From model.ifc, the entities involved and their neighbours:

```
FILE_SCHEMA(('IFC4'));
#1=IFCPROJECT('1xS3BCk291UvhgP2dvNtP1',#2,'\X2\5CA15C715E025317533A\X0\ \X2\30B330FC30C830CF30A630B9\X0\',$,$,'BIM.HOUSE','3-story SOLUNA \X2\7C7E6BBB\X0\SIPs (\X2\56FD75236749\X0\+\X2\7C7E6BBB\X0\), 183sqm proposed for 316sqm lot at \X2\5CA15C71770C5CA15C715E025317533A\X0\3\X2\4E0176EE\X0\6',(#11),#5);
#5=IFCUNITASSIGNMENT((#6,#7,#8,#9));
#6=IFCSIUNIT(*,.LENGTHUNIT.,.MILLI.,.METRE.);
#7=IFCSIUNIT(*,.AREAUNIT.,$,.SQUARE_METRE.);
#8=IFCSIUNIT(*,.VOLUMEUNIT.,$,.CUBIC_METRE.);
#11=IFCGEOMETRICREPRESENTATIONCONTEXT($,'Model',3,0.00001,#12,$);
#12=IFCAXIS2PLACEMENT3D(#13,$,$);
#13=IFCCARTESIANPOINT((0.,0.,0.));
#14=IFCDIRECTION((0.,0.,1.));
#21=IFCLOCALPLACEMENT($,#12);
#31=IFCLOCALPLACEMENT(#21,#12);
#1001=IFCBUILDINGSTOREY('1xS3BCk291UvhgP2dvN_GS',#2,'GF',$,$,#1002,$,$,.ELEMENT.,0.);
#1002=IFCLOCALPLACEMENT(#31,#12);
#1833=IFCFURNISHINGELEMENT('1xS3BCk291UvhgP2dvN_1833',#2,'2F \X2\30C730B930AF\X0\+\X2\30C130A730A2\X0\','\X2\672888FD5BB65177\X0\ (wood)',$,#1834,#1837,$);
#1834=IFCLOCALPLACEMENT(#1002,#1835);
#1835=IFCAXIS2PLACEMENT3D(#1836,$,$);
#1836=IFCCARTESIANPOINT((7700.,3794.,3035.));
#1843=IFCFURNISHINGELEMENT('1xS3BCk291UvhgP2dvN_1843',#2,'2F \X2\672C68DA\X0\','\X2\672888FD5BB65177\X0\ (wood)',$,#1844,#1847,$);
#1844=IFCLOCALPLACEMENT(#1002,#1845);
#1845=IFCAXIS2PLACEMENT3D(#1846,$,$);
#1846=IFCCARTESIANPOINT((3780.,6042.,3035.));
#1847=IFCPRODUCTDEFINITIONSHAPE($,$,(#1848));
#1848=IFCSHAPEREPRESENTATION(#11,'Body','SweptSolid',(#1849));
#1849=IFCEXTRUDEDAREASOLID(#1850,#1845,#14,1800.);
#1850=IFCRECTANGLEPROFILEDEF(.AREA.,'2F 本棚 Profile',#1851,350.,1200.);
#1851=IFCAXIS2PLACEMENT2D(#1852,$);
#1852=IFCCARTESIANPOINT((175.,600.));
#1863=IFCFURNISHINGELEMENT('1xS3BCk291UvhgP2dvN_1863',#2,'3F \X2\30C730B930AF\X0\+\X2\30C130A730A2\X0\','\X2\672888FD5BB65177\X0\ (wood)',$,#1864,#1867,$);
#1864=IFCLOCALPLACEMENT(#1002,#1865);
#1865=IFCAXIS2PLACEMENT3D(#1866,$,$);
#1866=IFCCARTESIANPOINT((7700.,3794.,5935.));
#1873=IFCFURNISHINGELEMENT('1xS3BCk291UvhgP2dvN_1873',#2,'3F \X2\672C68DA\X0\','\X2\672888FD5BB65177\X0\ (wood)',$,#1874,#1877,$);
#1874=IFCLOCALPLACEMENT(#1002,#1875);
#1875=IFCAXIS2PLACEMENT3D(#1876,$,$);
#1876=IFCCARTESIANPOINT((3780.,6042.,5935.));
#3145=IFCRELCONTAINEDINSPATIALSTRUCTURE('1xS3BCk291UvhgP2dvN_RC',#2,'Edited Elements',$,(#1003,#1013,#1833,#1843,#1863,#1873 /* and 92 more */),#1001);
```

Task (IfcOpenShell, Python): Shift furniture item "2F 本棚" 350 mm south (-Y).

```python
import ifcopenshell
import ifcopenshell.api.geometry
import ifcopenshell.util.placement

model = ifcopenshell.open("model.ifc")

item = model.by_guid("1xS3BCk291UvhgP2dvN_1843")
matrix = ifcopenshell.util.placement.get_local_placement(item.ObjectPlacement)
matrix[1, 3] -= 350.0
ifcopenshell.api.geometry.edit_object_placement(model, product=item, matrix=matrix, is_si=False)

print(ifcopenshell.util.placement.get_local_placement(item.ObjectPlacement).round(3) + 0.0)

model.write("model_v2.ifc")
```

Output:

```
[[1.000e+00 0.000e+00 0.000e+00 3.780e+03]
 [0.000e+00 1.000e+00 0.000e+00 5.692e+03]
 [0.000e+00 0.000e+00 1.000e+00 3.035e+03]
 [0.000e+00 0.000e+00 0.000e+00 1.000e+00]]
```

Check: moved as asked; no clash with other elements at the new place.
